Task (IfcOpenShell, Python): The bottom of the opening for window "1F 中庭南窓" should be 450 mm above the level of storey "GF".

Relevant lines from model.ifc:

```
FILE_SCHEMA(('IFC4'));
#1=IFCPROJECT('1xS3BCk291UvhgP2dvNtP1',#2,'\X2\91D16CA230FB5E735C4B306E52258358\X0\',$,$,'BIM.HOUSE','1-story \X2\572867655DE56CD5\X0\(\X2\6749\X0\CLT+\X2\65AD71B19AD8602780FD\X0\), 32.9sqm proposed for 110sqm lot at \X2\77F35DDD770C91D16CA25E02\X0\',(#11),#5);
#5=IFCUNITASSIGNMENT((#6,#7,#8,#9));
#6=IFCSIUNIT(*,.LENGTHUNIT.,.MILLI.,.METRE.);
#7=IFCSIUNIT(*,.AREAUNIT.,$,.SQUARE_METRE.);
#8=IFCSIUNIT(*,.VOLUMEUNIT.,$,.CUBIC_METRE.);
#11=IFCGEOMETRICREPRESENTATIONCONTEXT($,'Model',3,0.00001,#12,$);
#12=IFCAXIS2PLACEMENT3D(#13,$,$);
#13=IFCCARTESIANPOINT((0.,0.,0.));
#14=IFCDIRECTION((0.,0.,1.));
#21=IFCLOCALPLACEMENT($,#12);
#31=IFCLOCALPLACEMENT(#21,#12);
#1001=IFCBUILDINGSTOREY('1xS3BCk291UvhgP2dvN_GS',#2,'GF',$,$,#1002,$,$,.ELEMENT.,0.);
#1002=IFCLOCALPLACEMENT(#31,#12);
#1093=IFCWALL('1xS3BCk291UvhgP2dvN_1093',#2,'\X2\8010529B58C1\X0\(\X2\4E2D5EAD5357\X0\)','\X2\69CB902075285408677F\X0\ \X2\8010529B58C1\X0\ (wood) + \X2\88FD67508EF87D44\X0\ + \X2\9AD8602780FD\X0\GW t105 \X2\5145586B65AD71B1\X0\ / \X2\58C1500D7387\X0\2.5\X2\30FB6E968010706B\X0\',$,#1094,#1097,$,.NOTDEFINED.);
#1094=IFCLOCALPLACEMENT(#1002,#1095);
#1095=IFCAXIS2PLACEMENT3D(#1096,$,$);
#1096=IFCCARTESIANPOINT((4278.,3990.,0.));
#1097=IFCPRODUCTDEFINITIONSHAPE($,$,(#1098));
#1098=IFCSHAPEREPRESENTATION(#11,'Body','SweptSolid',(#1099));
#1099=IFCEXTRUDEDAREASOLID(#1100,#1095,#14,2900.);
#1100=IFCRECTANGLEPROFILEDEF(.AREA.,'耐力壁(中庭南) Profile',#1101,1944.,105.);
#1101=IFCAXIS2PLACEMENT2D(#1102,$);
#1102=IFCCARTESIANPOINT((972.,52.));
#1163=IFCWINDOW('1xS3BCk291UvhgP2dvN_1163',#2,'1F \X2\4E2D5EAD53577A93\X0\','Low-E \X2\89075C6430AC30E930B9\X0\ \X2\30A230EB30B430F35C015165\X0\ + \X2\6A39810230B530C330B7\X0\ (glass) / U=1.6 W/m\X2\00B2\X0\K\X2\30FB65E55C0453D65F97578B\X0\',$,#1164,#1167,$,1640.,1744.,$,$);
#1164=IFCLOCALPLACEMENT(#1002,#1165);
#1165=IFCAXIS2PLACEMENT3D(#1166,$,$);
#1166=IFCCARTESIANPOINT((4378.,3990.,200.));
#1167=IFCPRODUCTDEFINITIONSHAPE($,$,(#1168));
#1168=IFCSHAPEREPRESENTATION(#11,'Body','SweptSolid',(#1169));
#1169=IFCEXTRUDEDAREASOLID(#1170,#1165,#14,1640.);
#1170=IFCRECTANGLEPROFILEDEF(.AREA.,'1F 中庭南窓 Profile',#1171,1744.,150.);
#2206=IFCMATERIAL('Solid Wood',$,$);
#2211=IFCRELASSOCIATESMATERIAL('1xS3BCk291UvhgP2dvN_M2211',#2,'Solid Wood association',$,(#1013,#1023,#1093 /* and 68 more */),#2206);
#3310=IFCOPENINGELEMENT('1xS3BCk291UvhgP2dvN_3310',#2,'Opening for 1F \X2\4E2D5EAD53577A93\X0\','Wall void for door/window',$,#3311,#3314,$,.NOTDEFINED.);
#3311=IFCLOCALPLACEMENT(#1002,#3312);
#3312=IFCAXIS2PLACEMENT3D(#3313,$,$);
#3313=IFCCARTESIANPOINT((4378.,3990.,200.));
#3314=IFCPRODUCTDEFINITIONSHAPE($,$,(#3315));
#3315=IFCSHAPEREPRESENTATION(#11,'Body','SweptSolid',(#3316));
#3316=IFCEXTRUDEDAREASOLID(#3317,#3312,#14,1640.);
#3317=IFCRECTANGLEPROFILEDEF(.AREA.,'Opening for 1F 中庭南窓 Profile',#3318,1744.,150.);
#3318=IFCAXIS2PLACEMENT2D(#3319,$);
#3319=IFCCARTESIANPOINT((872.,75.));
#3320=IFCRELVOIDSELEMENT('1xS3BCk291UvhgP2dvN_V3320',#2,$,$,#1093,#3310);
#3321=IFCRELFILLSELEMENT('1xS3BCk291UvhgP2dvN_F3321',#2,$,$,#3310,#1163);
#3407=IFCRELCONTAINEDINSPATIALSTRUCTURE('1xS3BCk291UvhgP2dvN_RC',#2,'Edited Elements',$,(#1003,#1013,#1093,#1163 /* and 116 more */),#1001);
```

```python
import numpy as np
import ifcopenshell
import ifcopenshell.api.geometry
import ifcopenshell.geom
import ifcopenshell.util.element
import ifcopenshell.util.placement
import ifcopenshell.util.shape
import ifcopenshell.util.unit

model = ifcopenshell.open("model.ifc")
unit_scale = ifcopenshell.util.unit.calculate_unit_scale(model)

window = model.by_guid("1xS3BCk291UvhgP2dvN_1163")
opening = window.FillsVoids[0].RelatingOpeningElement
storey = ifcopenshell.util.element.get_container(window, ifc_class="IfcBuildingStorey")
level = ifcopenshell.util.placement.get_local_placement(storey.ObjectPlacement)[2, 3]

# The opening's origin need not be at the sill, so measure its lowest point.
shape = ifcopenshell.geom.create_shape(ifcopenshell.geom.settings(), opening)
bottom = ifcopenshell.util.shape.get_shape_bottom_elevation(shape, shape.geometry) / unit_scale
dz = level + 450.0 - bottom

shift = np.array([0.0, 0.0, dz])
# The window is not placed relative to its opening, so move both.
for product in (opening, window):
    matrix = ifcopenshell.util.placement.get_local_placement(product.ObjectPlacement)
    matrix[:3, 3] += shift
    ifcopenshell.api.geometry.edit_object_placement(model, product=product, matrix=matrix, is_si=False)

print(f"moved by {dz * unit_scale:+.3f} m")

model.write("model_updated.ifc")
```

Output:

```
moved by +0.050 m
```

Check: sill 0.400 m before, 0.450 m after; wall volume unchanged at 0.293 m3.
